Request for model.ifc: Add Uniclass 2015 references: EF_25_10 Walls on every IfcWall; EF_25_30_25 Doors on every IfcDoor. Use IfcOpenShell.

First a look at what the model holds.

```python
import ifcopenshell

model = ifcopenshell.open("model.ifc")
print(model.schema)
print("classifications:", [c.Name for c in model.by_type("IfcClassification")])
for ifc_class in ("IfcDoor", "IfcRoof", "IfcStair", "IfcWall", "IfcWindow"):
    print(ifc_class, len(model.by_type(ifc_class)))
```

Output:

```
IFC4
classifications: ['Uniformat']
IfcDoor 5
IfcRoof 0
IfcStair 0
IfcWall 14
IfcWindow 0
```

```python
import ifcopenshell
import ifcopenshell.api.classification

model = ifcopenshell.open("model.ifc")

system = ifcopenshell.api.classification.add_classification(model, classification="Uniclass 2015")

codes = {
    "IfcWall": ("EF_25_10", "Walls"),
    "IfcDoor": ("EF_25_30_25", "Doors"),
}
for ifc_class, (code, name) in codes.items():
    products = model.by_type(ifc_class)
    ifcopenshell.api.classification.add_reference(
        model, products=products, classification=system, identification=code, name=name
    )
    print(code, len(products))

model.write("model_v2.ifc")
```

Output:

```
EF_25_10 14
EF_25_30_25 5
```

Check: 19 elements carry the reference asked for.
